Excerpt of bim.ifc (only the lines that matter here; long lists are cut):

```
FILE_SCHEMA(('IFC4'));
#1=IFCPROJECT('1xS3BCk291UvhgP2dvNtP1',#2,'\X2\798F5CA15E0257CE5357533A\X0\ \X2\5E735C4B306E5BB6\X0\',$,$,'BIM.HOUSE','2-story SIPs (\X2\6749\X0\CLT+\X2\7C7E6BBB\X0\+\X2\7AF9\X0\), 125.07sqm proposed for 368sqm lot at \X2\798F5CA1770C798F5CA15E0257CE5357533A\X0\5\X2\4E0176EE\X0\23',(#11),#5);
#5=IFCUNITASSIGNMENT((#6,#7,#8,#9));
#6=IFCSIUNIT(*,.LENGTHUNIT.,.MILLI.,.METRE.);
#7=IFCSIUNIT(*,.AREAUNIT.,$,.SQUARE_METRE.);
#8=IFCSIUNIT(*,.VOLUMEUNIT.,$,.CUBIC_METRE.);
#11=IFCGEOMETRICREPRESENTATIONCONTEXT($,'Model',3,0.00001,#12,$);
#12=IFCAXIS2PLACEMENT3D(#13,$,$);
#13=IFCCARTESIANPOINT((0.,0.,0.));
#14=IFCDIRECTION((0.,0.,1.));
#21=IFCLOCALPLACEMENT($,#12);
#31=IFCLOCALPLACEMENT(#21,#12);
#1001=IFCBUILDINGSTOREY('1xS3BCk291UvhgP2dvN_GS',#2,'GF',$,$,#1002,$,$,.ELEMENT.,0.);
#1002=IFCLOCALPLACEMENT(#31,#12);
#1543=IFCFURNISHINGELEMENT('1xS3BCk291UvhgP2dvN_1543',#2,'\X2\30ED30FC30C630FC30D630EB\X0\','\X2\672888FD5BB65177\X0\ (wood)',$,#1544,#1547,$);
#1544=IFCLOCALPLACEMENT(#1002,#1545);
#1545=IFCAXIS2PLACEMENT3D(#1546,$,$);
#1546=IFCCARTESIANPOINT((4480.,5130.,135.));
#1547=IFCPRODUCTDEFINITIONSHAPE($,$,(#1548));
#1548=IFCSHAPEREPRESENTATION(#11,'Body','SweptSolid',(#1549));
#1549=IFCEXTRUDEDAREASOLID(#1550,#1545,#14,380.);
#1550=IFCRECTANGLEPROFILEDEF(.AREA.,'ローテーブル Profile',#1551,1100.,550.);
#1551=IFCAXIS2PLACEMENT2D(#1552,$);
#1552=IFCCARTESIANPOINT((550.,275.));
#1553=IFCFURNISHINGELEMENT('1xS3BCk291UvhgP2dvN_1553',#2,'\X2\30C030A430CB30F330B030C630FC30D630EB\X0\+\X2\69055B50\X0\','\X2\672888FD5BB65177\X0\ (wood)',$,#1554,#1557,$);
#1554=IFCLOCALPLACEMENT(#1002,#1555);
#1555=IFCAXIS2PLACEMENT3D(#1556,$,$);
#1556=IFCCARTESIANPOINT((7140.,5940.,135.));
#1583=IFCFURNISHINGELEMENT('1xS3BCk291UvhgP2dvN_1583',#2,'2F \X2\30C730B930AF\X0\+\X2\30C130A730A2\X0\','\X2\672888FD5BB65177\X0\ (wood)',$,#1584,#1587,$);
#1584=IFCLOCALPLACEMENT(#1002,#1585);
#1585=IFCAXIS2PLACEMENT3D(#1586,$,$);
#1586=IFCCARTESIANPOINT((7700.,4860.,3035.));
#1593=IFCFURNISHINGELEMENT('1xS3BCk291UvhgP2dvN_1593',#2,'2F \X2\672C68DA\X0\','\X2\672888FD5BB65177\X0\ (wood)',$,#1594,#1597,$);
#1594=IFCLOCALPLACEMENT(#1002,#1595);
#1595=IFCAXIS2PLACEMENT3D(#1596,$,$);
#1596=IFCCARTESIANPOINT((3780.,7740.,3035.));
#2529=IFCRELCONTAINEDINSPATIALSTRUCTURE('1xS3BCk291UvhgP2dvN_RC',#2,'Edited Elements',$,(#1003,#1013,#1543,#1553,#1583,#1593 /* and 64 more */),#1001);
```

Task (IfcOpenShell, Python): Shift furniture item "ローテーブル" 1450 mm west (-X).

```python
import ifcopenshell
import ifcopenshell.api.geometry
import ifcopenshell.util.placement

model = ifcopenshell.open("bim.ifc")

item = model.by_guid("1xS3BCk291UvhgP2dvN_1543")
matrix = ifcopenshell.util.placement.get_local_placement(item.ObjectPlacement)
matrix[0, 3] -= 1450.0
ifcopenshell.api.geometry.edit_object_placement(model, product=item, matrix=matrix, is_si=False)

print(ifcopenshell.util.placement.get_local_placement(item.ObjectPlacement).round(3) + 0.0)

model.write("bim_v2.ifc")
```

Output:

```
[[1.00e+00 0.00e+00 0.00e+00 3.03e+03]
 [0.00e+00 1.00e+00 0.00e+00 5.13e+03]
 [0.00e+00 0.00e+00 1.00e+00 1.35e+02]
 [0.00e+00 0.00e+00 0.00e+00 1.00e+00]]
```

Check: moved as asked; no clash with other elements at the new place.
